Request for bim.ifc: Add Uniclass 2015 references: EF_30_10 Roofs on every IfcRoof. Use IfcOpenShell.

First a look at what the model holds.

```python
import ifcopenshell

model = ifcopenshell.open("bim.ifc")
print(model.schema)
print("classifications:", [c.Name for c in model.by_type("IfcClassification")])
for ifc_class in ("IfcDoor", "IfcRoof", "IfcStair", "IfcWall", "IfcWindow"):
    print(ifc_class, len(model.by_type(ifc_class)))
```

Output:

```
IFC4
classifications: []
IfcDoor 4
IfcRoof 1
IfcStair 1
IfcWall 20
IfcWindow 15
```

```python
import ifcopenshell
import ifcopenshell.api.classification

model = ifcopenshell.open("bim.ifc")

system = ifcopenshell.api.classification.add_classification(model, classification="Uniclass 2015")

codes = {
    "IfcRoof": ("EF_30_10", "Roofs"),
}
for ifc_class, (code, name) in codes.items():
    products = model.by_type(ifc_class)
    ifcopenshell.api.classification.add_reference(
        model, products=products, classification=system, identification=code, name=name
    )
    print(code, len(products))

model.write("bim_v2.ifc")
```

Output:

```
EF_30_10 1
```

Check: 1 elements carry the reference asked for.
